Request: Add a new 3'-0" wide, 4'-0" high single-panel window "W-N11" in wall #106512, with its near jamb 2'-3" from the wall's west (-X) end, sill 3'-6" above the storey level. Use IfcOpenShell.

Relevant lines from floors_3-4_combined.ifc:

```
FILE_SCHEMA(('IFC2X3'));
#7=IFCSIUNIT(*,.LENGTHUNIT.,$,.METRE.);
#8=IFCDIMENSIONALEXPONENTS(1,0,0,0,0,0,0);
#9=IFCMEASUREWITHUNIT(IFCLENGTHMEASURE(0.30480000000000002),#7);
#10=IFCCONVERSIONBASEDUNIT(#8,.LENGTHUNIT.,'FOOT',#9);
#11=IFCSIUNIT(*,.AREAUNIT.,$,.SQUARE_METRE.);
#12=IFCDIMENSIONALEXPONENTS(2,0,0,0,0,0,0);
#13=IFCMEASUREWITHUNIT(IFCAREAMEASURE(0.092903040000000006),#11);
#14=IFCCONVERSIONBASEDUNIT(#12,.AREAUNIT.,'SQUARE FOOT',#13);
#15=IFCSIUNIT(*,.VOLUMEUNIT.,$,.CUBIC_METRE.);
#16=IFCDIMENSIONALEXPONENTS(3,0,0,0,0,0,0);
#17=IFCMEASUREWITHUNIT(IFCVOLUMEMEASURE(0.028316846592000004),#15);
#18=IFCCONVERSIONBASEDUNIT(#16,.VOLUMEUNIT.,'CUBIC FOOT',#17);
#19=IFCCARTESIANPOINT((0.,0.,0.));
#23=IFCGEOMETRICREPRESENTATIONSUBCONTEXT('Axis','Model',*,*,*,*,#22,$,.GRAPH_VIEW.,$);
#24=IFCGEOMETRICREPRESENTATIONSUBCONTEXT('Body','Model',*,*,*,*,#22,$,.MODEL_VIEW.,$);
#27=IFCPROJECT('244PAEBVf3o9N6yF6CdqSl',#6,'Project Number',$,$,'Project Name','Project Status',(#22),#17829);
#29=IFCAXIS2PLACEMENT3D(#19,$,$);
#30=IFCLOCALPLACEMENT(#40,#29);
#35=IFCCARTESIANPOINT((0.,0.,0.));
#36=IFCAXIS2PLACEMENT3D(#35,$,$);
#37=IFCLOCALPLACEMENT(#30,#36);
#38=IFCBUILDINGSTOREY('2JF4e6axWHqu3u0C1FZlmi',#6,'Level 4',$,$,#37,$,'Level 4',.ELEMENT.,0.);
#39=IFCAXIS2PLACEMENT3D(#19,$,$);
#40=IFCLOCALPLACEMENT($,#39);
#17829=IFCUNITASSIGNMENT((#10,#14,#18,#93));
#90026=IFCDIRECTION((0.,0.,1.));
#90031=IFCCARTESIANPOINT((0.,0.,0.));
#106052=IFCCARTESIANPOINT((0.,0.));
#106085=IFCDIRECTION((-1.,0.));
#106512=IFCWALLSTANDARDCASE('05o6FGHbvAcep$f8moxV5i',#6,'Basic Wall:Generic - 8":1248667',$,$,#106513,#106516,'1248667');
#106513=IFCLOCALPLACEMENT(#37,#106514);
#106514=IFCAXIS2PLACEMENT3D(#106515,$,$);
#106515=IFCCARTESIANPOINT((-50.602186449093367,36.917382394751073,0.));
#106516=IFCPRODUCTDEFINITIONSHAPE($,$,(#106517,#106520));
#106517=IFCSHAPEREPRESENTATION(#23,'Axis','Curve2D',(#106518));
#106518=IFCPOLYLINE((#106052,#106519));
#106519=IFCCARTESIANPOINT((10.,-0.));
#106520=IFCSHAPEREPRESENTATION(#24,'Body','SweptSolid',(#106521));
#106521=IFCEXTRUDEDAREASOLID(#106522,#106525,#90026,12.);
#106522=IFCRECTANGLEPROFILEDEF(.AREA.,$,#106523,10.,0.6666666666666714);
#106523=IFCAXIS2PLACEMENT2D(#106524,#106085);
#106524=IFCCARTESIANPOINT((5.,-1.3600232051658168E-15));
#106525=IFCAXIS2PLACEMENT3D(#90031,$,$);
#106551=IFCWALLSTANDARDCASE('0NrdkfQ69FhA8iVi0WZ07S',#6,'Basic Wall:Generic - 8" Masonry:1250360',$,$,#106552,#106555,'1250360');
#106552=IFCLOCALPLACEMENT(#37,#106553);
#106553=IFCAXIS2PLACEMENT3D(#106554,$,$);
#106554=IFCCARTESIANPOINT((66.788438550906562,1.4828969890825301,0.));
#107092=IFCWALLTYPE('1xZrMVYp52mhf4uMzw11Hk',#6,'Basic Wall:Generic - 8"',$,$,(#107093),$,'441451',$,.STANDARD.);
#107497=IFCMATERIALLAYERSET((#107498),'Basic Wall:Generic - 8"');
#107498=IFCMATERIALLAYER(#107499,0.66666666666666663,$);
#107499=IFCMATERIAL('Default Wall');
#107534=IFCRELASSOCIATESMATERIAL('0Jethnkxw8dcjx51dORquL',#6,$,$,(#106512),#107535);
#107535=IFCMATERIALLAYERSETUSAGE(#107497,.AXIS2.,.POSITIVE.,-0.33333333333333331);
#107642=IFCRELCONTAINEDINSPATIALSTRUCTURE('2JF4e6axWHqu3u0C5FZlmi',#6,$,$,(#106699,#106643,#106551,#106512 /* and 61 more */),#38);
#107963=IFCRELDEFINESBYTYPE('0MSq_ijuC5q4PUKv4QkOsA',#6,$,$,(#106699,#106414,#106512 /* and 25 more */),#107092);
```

```python
import numpy as np
import ifcopenshell
import ifcopenshell.api.feature
import ifcopenshell.api.geometry
import ifcopenshell.api.root
import ifcopenshell.api.spatial
import ifcopenshell.api.type
import ifcopenshell.geom
import ifcopenshell.util.element
import ifcopenshell.util.placement
import ifcopenshell.util.representation
import ifcopenshell.util.shape
import ifcopenshell.util.unit

model = ifcopenshell.open("floors_3-4_combined.ifc")
unit_scale = ifcopenshell.util.unit.calculate_unit_scale(model)
settings = ifcopenshell.geom.settings()


def volume(element):
    """Net volume in cubic metres, openings subtracted."""
    shape = ifcopenshell.geom.create_shape(settings, element)
    return ifcopenshell.util.shape.get_volume(shape.geometry)


wall = model.by_guid("05o6FGHbvAcep$f8moxV5i")
storey = ifcopenshell.util.element.get_container(wall, ifc_class="IfcBuildingStorey")
context = ifcopenshell.util.representation.get_context(model, "Model", "Body", "MODEL_VIEW")
before = volume(wall)

width, height, from_end, sill = 0.9144, 1.2192, 0.6858, 1.0668  # metres

# The wall runs along its own X axis, and the end named is its -X end.
wall_shape = ifcopenshell.geom.create_shape(settings, wall)
x, y, z = ifcopenshell.util.shape.get_vertices(wall_shape.geometry).T
start = x.min() + from_end
face, thickness = float(y.min()), float(y.max() - y.min())
wall_matrix = ifcopenshell.util.placement.get_local_placement(wall.ObjectPlacement)
level = ifcopenshell.util.placement.get_local_placement(storey.ObjectPlacement)[2, 3]


def in_wall(x, y):
    """Placement at x, y metres in the wall's axes, at sill height."""
    matrix = wall_matrix.copy()
    matrix[:, 3] = wall_matrix @ np.array([x / unit_scale, y / unit_scale, 0.0, 1.0])
    matrix[2, 3] = level + sill / unit_scale
    return matrix


# Opening: a box that overshoots both wall faces by 50 mm.
opening = ifcopenshell.api.root.create_entity(model, ifc_class="IfcOpeningElement")
box = ifcopenshell.api.geometry.add_wall_representation(
    model, context=context, length=width, height=height, thickness=thickness + 0.1
)
ifcopenshell.api.geometry.assign_representation(model, product=opening, representation=box)
ifcopenshell.api.geometry.edit_object_placement(model, product=opening, matrix=in_wall(start, face - 0.05), is_si=False)
ifcopenshell.api.feature.add_feature(model, feature=opening, element=wall)

window = ifcopenshell.api.root.create_entity(model, ifc_class="IfcWindow", name="W-N11")
window.OverallWidth, window.OverallHeight = width / unit_scale, height / unit_scale
body = ifcopenshell.api.geometry.add_window_representation(
    model,
    context=context,
    overall_width=window.OverallWidth,
    overall_height=window.OverallHeight,
    partition_type="SINGLE_PANEL",
)
ifcopenshell.api.geometry.assign_representation(model, product=window, representation=body)
ifcopenshell.api.spatial.assign_container(model, products=[window], relating_structure=storey)
fills = ifcopenshell.api.feature.add_filling(model, opening=opening, element=window)
fills.OwnerHistory = window.OwnerHistory  # required in IFC2X3

# IFC2X3 keeps the operation on the window style.
style = ifcopenshell.api.root.create_entity(model, ifc_class="IfcWindowStyle", name="W-N11")
style.OperationType, style.ConstructionType = "SINGLE_PANEL", "NOTDEFINED"
style.ParameterTakesPrecedence = style.Sizeable = False
ifcopenshell.api.type.assign_type(model, related_objects=[window], relating_type=style)

# Centre the window in the wall's thickness.
ifcopenshell.api.geometry.edit_object_placement(model, product=window, matrix=in_wall(start, face), is_si=False)
window_shape = ifcopenshell.geom.create_shape(settings, window)
depth = ifcopenshell.util.shape.get_vertices(window_shape.geometry)[:, 1]
offset = face + thickness / 2 - (depth.min() + depth.max()) / 2
ifcopenshell.api.geometry.edit_object_placement(model, product=window, matrix=in_wall(start, offset), is_si=False)

after = volume(wall)

print(f"wall volume {before:.3f} -> {after:.3f} m3")

model.write("floors_3-4_combined_v2.ifc")
```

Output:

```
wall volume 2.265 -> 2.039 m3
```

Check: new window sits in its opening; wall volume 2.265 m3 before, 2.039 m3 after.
